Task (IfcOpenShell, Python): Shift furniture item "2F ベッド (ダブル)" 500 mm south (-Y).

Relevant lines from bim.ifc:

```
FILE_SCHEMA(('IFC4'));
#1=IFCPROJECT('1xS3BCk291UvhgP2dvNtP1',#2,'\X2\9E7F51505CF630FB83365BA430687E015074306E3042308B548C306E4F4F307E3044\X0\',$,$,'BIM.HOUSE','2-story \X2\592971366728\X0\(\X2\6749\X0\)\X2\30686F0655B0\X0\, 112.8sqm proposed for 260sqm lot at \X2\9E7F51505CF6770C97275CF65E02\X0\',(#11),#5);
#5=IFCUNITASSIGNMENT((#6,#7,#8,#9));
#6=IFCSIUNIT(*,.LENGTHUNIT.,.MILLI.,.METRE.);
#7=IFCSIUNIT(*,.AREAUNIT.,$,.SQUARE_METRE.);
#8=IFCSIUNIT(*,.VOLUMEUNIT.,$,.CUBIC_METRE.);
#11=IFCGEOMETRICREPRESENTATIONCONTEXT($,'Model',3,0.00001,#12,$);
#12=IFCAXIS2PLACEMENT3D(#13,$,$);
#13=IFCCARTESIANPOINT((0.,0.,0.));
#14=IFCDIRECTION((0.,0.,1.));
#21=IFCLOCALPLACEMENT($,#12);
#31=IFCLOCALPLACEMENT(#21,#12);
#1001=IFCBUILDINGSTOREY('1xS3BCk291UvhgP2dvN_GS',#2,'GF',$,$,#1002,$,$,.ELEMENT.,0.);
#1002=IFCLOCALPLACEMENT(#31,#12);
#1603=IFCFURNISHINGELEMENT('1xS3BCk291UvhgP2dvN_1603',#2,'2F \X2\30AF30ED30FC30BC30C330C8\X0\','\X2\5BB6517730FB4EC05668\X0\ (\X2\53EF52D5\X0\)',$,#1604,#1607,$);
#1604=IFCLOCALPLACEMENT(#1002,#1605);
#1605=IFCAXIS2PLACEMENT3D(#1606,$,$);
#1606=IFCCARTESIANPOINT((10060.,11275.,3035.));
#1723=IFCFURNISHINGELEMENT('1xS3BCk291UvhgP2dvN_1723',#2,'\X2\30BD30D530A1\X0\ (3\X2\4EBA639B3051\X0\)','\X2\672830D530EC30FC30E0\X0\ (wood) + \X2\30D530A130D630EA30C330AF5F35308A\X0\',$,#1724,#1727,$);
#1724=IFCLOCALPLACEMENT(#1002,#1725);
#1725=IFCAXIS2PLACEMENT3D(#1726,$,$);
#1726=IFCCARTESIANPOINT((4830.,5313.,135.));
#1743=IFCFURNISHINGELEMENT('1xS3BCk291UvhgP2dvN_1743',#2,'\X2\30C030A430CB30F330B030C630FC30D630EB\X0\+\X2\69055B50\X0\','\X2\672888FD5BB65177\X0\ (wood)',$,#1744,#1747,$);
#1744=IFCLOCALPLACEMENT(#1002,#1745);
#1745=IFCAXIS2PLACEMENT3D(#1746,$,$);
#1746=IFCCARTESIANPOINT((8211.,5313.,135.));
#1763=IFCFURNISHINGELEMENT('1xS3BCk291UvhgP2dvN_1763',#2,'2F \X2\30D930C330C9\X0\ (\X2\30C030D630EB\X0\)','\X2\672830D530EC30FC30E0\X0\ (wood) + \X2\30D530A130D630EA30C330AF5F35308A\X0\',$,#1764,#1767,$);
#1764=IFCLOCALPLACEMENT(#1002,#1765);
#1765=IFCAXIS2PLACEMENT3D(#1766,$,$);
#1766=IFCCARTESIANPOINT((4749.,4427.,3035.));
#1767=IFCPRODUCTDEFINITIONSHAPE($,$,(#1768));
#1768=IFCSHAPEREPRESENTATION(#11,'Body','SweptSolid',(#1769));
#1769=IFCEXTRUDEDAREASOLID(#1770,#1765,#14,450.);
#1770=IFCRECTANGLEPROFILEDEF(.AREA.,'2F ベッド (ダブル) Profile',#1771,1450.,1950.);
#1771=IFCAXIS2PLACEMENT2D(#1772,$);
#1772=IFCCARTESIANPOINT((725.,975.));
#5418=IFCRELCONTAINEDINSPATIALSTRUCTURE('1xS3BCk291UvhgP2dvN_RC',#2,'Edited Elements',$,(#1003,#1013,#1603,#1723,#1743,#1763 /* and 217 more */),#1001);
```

```python
import ifcopenshell
import ifcopenshell.api.geometry
import ifcopenshell.util.placement
import ifcopenshell.util.unit

model = ifcopenshell.open("bim.ifc")
unit_scale = ifcopenshell.util.unit.calculate_unit_scale(model)

item = model.by_guid("1xS3BCk291UvhgP2dvN_1763")
matrix = ifcopenshell.util.placement.get_local_placement(item.ObjectPlacement)
matrix[1, 3] -= 0.5 / unit_scale
ifcopenshell.api.geometry.edit_object_placement(model, product=item, matrix=matrix, is_si=False)

print(ifcopenshell.util.placement.get_local_placement(item.ObjectPlacement).round(3) + 0.0)

model.write("bim_v2.ifc")
```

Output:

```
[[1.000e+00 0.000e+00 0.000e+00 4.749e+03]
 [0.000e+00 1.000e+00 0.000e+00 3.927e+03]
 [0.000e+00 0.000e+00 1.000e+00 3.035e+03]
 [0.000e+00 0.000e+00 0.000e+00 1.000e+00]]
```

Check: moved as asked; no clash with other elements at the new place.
